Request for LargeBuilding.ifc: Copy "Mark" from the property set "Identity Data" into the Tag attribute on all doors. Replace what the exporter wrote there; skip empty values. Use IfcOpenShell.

First a look at what the model holds.

```python
import ifcopenshell
import ifcopenshell.util.element

model = ifcopenshell.open("LargeBuilding.ifc")
print(model.schema)
doors = model.by_type("IfcDoor")
print(len(doors), "doors")
for e in doors[:8]:
    source = ifcopenshell.util.element.get_pset(e, "Identity Data", "Mark")
    target = e.Tag
    print(e.id(), repr(source), repr(target), sep=" | ")
```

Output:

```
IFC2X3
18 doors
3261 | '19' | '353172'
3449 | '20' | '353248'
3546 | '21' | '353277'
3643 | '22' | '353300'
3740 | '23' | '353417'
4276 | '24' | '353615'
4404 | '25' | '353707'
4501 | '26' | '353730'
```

```python
import ifcopenshell
import ifcopenshell.util.element

model = ifcopenshell.open("LargeBuilding.ifc")

count = 0
for e in model.by_type("IfcDoor"):
    value = ifcopenshell.util.element.get_pset(e, "Identity Data", "Mark")
    current = e.Tag
    if not value or not value.strip() or current == value:
        continue
    e.Tag = value
    count += 1

print(count, "doors updated")

model.write("LargeBuilding_rev.ifc")
```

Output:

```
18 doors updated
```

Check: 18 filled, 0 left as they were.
